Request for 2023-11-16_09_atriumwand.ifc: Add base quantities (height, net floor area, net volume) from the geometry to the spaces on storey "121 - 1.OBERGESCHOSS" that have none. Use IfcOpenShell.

First a look at what the model holds.

```python
import ifcopenshell
import ifcopenshell.util.element
import ifcopenshell.util.unit

model = ifcopenshell.open("2023-11-16_09_atriumwand.ifc")
print(model.schema)
for unit_type in ("LENGTHUNIT", "AREAUNIT", "VOLUMEUNIT"):
    print(unit_type, ifcopenshell.util.unit.calculate_unit_scale(model, unit_type))
storey = next(s for s in model.by_type("IfcBuildingStorey") if s.Name == "121 - 1.OBERGESCHOSS")
spaces = [e for e in ifcopenshell.util.element.get_decomposition(storey) if e.is_a("IfcSpace")]
for e in sorted(spaces, key=lambda e: e.id()):
    print(e.id(), e.is_a(), e.Name, list(ifcopenshell.util.element.get_psets(e, qtos_only=True)), sep=" | ")
```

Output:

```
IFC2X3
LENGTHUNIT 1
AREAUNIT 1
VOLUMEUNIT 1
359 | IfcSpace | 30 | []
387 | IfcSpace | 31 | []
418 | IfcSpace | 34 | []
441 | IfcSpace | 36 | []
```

```python
import ifcopenshell
import ifcopenshell.api.pset
import ifcopenshell.geom
import ifcopenshell.util.element
import ifcopenshell.util.shape
import ifcopenshell.util.unit

model = ifcopenshell.open("2023-11-16_09_atriumwand.ifc")
unit_scale = ifcopenshell.util.unit.calculate_unit_scale(model)
area_scale = ifcopenshell.util.unit.calculate_unit_scale(model, "AREAUNIT")
volume_scale = ifcopenshell.util.unit.calculate_unit_scale(model, "VOLUMEUNIT")
settings = ifcopenshell.geom.settings()

storey = next(s for s in model.by_type("IfcBuildingStorey") if s.Name == "121 - 1.OBERGESCHOSS")
spaces = [e for e in ifcopenshell.util.element.get_decomposition(storey) if e.is_a("IfcSpace")]

for e in sorted(spaces, key=lambda e: e.id()):
    if ifcopenshell.util.element.get_psets(e, qtos_only=True, should_inherit=False):
        continue
    # Geometry comes back in metres, in the element's own axes.
    shape = ifcopenshell.geom.create_shape(settings, e)
    values = {
        "Height": ifcopenshell.util.shape.get_z(shape.geometry) / unit_scale,
        "NetFloorArea": ifcopenshell.util.shape.get_footprint_area(shape.geometry) / area_scale,
        "NetVolume": ifcopenshell.util.shape.get_volume(shape.geometry) / volume_scale,
    }
    qto = ifcopenshell.api.pset.add_qto(model, product=e, name="BaseQuantities")
    ifcopenshell.api.pset.edit_qto(model, qto=qto, properties=values)
    print(e.id(), {k: round(v, 3) for k, v in values.items()})

model.write("2023-11-16_09_atriumwand_rev.ifc")
```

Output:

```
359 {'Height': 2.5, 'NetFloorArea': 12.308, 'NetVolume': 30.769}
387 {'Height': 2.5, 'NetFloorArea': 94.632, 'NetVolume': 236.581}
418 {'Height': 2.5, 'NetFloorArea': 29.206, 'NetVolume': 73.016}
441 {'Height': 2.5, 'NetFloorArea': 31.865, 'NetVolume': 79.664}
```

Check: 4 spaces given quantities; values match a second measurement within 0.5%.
